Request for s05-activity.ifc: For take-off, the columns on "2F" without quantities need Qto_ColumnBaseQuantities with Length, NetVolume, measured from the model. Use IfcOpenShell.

First a look at what the model holds.

```python
import ifcopenshell
import ifcopenshell.util.element
import ifcopenshell.util.unit

model = ifcopenshell.open("s05-activity.ifc")
print(model.schema)
for unit_type in ("LENGTHUNIT", "AREAUNIT", "VOLUMEUNIT"):
    print(unit_type, ifcopenshell.util.unit.calculate_unit_scale(model, unit_type))
storey = next(s for s in model.by_type("IfcBuildingStorey") if s.Name == "2F")
columns = [e for e in ifcopenshell.util.element.get_decomposition(storey) if e.is_a("IfcColumn")]
for e in sorted(columns, key=lambda e: e.id()):
    print(e.id(), e.is_a(), e.Name, list(ifcopenshell.util.element.get_psets(e, qtos_only=True)), sep=" | ")
```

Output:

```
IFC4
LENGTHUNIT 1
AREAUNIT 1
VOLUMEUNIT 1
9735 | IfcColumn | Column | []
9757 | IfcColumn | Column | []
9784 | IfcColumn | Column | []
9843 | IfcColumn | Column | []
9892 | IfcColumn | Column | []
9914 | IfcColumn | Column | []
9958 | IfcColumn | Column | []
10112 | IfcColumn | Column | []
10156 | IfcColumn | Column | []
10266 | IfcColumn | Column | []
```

```python
import ifcopenshell
import ifcopenshell.api.pset
import ifcopenshell.geom
import ifcopenshell.util.element
import ifcopenshell.util.shape
import ifcopenshell.util.unit

model = ifcopenshell.open("s05-activity.ifc")
unit_scale = ifcopenshell.util.unit.calculate_unit_scale(model)
volume_scale = ifcopenshell.util.unit.calculate_unit_scale(model, "VOLUMEUNIT")
settings = ifcopenshell.geom.settings()

storey = next(s for s in model.by_type("IfcBuildingStorey") if s.Name == "2F")
columns = [e for e in ifcopenshell.util.element.get_decomposition(storey) if e.is_a("IfcColumn")]

for e in sorted(columns, key=lambda e: e.id()):
    if ifcopenshell.util.element.get_psets(e, qtos_only=True, should_inherit=False):
        continue
    # Geometry comes back in metres, in the element's own axes.
    shape = ifcopenshell.geom.create_shape(settings, e)
    values = {
        "Length": ifcopenshell.util.shape.get_z(shape.geometry) / unit_scale,
        "NetVolume": ifcopenshell.util.shape.get_volume(shape.geometry) / volume_scale,
    }
    qto = ifcopenshell.api.pset.add_qto(model, product=e, name="Qto_ColumnBaseQuantities")
    ifcopenshell.api.pset.edit_qto(model, qto=qto, properties=values)
    print(e.id(), {k: round(v, 3) for k, v in values.items()})

model.write("s05-activity_edited.ifc")
```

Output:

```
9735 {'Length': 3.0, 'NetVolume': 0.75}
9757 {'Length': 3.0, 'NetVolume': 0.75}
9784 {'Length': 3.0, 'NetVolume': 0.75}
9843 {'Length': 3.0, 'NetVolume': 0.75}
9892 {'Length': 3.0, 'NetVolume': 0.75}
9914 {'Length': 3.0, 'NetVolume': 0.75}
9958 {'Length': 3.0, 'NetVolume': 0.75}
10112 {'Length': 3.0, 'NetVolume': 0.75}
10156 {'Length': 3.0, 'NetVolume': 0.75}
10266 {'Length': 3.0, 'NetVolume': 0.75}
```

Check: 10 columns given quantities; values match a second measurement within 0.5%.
